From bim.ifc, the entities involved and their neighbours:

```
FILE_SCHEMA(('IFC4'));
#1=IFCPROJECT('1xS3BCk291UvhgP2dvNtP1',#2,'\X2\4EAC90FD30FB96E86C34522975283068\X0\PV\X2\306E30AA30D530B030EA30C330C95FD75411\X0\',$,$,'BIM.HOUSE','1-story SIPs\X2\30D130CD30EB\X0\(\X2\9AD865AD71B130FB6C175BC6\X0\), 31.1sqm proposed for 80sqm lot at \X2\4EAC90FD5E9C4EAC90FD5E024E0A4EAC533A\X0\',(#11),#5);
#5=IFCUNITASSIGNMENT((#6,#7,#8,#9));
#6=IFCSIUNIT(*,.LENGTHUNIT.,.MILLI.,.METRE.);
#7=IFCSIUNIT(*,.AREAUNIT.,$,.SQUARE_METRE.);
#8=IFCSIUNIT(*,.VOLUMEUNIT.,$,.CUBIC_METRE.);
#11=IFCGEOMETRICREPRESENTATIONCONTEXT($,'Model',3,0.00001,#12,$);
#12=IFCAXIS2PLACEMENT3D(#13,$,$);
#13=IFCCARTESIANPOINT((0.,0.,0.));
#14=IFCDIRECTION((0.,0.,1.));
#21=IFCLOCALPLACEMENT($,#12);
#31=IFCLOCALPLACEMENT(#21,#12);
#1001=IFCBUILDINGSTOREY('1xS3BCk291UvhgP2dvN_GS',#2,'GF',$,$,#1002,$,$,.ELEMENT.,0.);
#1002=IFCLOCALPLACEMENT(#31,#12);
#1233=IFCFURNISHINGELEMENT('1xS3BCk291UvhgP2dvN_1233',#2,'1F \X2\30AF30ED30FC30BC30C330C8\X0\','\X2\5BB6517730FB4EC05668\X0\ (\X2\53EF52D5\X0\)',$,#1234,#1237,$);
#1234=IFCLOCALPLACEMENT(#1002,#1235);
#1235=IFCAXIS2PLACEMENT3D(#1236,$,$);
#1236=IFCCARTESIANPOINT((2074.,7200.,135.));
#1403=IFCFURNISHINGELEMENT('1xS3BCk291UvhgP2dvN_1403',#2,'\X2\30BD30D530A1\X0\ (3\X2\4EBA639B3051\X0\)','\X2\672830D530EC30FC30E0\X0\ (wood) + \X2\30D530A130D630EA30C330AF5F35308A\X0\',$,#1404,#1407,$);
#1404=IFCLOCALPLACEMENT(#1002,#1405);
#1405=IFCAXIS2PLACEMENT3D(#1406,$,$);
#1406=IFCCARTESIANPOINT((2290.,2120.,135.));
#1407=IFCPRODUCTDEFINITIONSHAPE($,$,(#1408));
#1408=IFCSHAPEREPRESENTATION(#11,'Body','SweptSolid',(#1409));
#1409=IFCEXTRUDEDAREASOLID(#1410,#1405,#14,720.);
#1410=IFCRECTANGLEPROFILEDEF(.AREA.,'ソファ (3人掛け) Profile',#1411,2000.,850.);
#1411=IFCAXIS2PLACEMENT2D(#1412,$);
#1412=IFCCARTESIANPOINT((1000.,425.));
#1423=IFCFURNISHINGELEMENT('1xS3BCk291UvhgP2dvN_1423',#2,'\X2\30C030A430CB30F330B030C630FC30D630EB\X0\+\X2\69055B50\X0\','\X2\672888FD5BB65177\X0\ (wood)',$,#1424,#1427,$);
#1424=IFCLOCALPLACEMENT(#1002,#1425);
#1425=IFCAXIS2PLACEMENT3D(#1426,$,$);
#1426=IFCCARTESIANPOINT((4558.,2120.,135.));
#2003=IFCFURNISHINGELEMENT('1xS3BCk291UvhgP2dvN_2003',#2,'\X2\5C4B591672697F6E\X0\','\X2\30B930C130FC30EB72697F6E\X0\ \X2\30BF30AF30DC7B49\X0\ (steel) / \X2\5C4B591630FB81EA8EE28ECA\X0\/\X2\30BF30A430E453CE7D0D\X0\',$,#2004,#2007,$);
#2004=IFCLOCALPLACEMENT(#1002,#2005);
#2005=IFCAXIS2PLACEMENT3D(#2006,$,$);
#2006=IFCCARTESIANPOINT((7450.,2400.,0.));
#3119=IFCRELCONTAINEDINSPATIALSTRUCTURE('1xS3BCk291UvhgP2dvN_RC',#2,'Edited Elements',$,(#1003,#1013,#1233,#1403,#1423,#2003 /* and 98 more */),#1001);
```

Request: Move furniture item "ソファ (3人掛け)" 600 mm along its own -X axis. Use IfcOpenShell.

```python
import ifcopenshell
import ifcopenshell.api.geometry
import ifcopenshell.util.placement
import ifcopenshell.util.unit

model = ifcopenshell.open("bim.ifc")
unit_scale = ifcopenshell.util.unit.calculate_unit_scale(model)

item = model.by_guid("1xS3BCk291UvhgP2dvN_1403")
matrix = ifcopenshell.util.placement.get_local_placement(item.ObjectPlacement)
matrix[:3, 3] -= matrix[:3, 0] * 0.6 / unit_scale
ifcopenshell.api.geometry.edit_object_placement(model, product=item, matrix=matrix, is_si=False)

print(ifcopenshell.util.placement.get_local_placement(item.ObjectPlacement).round(3) + 0.0)

model.write("bim_rev.ifc")
```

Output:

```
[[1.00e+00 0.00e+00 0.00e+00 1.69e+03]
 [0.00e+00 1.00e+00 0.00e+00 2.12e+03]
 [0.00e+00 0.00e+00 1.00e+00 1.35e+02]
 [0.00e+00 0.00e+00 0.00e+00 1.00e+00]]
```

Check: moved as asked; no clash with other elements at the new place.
